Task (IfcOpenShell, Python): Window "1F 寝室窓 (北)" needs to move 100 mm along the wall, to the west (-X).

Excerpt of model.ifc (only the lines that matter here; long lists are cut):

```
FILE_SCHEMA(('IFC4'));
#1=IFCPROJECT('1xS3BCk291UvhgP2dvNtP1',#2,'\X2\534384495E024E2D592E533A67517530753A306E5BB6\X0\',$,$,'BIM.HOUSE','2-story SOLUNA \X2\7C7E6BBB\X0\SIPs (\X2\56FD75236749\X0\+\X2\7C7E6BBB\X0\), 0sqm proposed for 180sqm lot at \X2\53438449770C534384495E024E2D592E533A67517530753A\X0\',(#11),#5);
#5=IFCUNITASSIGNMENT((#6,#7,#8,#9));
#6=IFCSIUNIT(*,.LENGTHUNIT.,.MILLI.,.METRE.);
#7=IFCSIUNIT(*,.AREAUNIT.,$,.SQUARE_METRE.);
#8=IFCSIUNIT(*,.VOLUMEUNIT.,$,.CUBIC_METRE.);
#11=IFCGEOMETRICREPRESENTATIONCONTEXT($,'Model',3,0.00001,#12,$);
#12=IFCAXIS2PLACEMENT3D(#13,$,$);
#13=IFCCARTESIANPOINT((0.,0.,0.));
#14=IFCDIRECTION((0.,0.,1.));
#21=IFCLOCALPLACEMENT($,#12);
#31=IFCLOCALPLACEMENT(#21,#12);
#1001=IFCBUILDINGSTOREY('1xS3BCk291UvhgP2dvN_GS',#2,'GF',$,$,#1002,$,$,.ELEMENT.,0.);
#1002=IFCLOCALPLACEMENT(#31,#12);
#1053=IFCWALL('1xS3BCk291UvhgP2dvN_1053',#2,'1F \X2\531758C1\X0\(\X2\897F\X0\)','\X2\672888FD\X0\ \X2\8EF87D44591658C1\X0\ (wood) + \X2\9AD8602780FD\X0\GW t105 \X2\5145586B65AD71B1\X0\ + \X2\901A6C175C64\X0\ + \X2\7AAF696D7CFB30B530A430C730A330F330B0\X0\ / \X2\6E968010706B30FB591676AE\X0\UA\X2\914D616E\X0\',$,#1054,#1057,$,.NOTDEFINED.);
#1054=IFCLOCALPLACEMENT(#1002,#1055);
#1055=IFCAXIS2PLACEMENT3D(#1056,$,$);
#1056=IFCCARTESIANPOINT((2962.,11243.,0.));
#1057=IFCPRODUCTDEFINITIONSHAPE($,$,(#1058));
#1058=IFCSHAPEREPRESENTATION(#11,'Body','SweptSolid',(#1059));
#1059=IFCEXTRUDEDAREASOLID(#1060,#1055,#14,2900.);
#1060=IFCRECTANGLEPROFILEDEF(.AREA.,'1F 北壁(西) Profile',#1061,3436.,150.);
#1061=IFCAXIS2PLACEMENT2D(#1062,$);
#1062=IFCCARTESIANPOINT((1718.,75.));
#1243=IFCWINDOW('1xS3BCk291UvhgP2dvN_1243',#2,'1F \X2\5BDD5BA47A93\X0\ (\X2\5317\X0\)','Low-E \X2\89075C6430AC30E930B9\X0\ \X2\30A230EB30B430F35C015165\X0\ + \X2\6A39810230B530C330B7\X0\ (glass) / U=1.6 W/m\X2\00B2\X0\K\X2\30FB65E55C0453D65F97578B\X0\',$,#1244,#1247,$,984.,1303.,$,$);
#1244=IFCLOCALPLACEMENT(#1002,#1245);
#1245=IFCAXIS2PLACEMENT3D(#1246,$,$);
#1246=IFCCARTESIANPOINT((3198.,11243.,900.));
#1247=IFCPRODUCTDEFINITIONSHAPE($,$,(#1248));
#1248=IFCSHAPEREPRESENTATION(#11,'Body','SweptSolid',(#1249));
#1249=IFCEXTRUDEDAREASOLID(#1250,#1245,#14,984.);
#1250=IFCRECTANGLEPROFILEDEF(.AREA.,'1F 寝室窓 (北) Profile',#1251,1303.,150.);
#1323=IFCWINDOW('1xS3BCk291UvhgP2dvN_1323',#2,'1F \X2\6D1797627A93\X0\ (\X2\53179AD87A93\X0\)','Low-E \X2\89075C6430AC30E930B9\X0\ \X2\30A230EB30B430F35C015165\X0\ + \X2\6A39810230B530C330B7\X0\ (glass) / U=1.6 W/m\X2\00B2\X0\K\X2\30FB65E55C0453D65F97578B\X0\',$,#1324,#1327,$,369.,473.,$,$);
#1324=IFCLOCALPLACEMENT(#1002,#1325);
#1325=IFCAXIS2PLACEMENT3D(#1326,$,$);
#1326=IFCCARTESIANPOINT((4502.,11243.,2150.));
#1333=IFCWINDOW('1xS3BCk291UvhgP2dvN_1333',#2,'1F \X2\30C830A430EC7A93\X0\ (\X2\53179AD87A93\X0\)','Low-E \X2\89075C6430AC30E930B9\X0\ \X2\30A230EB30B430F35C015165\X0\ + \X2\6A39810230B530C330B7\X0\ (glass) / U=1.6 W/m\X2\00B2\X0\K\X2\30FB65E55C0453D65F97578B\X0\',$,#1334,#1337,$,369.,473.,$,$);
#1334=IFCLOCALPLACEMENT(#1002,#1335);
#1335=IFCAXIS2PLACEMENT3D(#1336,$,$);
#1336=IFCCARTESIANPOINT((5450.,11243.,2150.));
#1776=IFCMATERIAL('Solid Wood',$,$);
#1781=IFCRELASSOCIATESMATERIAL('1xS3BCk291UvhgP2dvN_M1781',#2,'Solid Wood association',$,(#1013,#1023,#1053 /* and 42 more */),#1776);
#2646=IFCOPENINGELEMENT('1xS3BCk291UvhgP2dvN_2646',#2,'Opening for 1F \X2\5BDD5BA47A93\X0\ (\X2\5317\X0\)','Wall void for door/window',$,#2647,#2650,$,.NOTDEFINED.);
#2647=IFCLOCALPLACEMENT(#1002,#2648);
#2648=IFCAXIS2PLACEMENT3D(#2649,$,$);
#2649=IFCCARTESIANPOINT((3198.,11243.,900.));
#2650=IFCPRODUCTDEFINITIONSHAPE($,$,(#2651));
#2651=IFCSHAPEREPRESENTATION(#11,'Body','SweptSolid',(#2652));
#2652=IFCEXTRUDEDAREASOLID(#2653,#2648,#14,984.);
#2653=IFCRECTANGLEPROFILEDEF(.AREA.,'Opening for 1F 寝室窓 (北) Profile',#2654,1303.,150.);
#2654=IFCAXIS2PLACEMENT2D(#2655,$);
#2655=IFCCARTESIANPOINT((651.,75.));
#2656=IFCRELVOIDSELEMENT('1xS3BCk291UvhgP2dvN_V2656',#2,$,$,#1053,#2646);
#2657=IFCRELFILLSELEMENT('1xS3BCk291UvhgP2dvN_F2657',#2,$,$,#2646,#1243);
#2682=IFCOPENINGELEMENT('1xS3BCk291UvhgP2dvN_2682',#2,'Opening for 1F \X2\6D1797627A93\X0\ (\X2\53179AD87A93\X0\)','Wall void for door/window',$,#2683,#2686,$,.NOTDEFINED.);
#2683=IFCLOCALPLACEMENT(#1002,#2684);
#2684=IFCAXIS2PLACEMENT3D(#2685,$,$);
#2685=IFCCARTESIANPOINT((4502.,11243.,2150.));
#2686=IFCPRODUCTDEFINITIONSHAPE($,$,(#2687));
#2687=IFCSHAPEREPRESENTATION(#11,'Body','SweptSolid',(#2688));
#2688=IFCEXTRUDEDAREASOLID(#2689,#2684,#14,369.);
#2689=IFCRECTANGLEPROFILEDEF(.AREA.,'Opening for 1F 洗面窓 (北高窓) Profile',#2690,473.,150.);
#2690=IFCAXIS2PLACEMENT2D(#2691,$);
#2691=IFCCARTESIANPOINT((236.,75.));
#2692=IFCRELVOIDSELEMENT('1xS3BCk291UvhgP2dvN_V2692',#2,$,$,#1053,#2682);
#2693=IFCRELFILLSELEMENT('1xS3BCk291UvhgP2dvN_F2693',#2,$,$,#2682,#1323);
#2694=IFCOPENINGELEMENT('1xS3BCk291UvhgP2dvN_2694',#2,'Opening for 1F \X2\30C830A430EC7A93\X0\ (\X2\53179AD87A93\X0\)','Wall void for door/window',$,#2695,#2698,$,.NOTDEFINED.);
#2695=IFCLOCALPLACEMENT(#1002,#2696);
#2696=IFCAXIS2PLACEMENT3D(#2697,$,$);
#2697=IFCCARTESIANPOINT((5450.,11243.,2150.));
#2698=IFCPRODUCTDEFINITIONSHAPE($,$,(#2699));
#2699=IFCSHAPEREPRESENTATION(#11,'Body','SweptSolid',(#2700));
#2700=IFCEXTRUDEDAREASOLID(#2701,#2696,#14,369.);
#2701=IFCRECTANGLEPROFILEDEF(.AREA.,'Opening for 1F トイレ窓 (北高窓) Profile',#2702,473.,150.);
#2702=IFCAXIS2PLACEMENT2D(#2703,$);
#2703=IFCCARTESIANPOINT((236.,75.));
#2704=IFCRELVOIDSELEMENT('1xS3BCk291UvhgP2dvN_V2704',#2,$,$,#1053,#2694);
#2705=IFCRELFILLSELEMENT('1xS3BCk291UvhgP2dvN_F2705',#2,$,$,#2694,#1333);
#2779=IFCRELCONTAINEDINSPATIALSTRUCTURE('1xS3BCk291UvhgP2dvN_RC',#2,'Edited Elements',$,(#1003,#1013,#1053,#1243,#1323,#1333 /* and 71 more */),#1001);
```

```python
import ifcopenshell
import ifcopenshell.api.geometry
import ifcopenshell.util.placement
import ifcopenshell.util.unit

model = ifcopenshell.open("model.ifc")
unit_scale = ifcopenshell.util.unit.calculate_unit_scale(model)

window = model.by_guid("1xS3BCk291UvhgP2dvN_1243")
opening = window.FillsVoids[0].RelatingOpeningElement
wall = opening.VoidsElements[0].RelatingBuildingElement

wall_matrix = ifcopenshell.util.placement.get_local_placement(wall.ObjectPlacement)
shift = wall_matrix[:3, 0] * -0.1 / unit_scale
before = ifcopenshell.util.placement.get_local_placement(window.ObjectPlacement)[:3, 3].copy()

# The window is not placed relative to its opening, so move both.
for product in (opening, window):
    matrix = ifcopenshell.util.placement.get_local_placement(product.ObjectPlacement)
    matrix[:3, 3] += shift
    ifcopenshell.api.geometry.edit_object_placement(model, product=product, matrix=matrix, is_si=False)

after = ifcopenshell.util.placement.get_local_placement(window.ObjectPlacement)[:3, 3]
print("window moved by", (after - before).round(3) + 0.0)

model.write("model_updated.ifc")
```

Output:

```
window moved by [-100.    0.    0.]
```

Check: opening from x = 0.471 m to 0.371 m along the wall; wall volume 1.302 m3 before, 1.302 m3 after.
